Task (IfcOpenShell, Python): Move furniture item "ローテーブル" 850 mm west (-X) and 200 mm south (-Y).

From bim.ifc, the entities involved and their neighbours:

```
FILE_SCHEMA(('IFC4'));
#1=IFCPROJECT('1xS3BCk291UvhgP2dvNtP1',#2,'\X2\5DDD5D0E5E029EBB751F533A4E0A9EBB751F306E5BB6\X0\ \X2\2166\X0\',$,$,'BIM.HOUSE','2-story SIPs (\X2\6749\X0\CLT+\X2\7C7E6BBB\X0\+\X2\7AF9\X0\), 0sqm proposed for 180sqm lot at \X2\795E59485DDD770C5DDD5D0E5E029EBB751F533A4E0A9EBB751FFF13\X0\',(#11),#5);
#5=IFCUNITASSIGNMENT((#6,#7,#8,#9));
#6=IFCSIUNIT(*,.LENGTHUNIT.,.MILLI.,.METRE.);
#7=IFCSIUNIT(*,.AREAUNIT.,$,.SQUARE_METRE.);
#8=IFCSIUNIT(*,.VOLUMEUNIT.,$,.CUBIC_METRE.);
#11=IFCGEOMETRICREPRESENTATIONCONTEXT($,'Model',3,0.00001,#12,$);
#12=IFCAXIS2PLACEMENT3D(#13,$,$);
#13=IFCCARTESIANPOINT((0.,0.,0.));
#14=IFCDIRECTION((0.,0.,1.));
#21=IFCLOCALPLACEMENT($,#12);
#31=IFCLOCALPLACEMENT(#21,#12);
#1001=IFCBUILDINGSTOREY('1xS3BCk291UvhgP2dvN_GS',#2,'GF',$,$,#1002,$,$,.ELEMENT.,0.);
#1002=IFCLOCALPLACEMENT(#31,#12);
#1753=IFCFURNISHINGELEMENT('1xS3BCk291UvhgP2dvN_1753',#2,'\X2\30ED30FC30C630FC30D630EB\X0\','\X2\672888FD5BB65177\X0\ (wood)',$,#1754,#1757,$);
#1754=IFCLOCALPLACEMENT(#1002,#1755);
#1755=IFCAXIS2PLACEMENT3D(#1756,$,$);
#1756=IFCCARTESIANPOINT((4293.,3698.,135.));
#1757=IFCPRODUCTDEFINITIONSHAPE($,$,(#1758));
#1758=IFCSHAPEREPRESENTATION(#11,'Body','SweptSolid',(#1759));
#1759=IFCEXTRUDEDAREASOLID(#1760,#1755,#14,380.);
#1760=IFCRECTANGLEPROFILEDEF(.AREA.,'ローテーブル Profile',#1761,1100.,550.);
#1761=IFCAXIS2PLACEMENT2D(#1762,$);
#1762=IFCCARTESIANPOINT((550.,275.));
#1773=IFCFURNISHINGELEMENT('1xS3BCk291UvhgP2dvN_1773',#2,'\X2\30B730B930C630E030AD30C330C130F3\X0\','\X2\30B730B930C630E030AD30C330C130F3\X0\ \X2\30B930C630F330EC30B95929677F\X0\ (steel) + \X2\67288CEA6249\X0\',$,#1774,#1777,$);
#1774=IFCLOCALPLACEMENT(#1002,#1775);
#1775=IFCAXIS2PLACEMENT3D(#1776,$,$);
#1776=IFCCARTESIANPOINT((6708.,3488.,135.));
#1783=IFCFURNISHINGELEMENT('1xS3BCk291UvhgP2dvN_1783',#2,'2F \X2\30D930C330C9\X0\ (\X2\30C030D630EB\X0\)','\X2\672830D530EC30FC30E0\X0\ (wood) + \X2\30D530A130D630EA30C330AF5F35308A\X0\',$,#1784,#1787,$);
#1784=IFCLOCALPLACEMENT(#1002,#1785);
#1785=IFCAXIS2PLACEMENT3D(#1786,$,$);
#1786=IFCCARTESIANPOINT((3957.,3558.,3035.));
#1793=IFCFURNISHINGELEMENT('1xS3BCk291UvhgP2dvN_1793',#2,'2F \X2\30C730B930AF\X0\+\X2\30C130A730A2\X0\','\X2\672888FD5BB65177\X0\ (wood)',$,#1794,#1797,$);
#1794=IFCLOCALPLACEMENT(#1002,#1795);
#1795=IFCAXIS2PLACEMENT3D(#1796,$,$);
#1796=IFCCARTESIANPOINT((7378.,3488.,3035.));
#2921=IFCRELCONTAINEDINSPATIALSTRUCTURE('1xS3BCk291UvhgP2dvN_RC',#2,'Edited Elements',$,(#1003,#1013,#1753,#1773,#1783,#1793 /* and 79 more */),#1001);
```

```python
import ifcopenshell
import ifcopenshell.api.geometry
import ifcopenshell.util.placement
import ifcopenshell.util.unit

model = ifcopenshell.open("bim.ifc")
unit_scale = ifcopenshell.util.unit.calculate_unit_scale(model)

item = model.by_guid("1xS3BCk291UvhgP2dvN_1753")
matrix = ifcopenshell.util.placement.get_local_placement(item.ObjectPlacement)
matrix[0, 3] -= 0.85 / unit_scale
matrix[1, 3] -= 0.2 / unit_scale
ifcopenshell.api.geometry.edit_object_placement(model, product=item, matrix=matrix, is_si=False)

print(ifcopenshell.util.placement.get_local_placement(item.ObjectPlacement).round(3) + 0.0)

model.write("bim_updated.ifc")
```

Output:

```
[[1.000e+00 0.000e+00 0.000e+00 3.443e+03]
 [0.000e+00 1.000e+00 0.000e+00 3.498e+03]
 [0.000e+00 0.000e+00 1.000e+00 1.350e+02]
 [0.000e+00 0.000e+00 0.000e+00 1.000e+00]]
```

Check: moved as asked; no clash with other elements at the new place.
